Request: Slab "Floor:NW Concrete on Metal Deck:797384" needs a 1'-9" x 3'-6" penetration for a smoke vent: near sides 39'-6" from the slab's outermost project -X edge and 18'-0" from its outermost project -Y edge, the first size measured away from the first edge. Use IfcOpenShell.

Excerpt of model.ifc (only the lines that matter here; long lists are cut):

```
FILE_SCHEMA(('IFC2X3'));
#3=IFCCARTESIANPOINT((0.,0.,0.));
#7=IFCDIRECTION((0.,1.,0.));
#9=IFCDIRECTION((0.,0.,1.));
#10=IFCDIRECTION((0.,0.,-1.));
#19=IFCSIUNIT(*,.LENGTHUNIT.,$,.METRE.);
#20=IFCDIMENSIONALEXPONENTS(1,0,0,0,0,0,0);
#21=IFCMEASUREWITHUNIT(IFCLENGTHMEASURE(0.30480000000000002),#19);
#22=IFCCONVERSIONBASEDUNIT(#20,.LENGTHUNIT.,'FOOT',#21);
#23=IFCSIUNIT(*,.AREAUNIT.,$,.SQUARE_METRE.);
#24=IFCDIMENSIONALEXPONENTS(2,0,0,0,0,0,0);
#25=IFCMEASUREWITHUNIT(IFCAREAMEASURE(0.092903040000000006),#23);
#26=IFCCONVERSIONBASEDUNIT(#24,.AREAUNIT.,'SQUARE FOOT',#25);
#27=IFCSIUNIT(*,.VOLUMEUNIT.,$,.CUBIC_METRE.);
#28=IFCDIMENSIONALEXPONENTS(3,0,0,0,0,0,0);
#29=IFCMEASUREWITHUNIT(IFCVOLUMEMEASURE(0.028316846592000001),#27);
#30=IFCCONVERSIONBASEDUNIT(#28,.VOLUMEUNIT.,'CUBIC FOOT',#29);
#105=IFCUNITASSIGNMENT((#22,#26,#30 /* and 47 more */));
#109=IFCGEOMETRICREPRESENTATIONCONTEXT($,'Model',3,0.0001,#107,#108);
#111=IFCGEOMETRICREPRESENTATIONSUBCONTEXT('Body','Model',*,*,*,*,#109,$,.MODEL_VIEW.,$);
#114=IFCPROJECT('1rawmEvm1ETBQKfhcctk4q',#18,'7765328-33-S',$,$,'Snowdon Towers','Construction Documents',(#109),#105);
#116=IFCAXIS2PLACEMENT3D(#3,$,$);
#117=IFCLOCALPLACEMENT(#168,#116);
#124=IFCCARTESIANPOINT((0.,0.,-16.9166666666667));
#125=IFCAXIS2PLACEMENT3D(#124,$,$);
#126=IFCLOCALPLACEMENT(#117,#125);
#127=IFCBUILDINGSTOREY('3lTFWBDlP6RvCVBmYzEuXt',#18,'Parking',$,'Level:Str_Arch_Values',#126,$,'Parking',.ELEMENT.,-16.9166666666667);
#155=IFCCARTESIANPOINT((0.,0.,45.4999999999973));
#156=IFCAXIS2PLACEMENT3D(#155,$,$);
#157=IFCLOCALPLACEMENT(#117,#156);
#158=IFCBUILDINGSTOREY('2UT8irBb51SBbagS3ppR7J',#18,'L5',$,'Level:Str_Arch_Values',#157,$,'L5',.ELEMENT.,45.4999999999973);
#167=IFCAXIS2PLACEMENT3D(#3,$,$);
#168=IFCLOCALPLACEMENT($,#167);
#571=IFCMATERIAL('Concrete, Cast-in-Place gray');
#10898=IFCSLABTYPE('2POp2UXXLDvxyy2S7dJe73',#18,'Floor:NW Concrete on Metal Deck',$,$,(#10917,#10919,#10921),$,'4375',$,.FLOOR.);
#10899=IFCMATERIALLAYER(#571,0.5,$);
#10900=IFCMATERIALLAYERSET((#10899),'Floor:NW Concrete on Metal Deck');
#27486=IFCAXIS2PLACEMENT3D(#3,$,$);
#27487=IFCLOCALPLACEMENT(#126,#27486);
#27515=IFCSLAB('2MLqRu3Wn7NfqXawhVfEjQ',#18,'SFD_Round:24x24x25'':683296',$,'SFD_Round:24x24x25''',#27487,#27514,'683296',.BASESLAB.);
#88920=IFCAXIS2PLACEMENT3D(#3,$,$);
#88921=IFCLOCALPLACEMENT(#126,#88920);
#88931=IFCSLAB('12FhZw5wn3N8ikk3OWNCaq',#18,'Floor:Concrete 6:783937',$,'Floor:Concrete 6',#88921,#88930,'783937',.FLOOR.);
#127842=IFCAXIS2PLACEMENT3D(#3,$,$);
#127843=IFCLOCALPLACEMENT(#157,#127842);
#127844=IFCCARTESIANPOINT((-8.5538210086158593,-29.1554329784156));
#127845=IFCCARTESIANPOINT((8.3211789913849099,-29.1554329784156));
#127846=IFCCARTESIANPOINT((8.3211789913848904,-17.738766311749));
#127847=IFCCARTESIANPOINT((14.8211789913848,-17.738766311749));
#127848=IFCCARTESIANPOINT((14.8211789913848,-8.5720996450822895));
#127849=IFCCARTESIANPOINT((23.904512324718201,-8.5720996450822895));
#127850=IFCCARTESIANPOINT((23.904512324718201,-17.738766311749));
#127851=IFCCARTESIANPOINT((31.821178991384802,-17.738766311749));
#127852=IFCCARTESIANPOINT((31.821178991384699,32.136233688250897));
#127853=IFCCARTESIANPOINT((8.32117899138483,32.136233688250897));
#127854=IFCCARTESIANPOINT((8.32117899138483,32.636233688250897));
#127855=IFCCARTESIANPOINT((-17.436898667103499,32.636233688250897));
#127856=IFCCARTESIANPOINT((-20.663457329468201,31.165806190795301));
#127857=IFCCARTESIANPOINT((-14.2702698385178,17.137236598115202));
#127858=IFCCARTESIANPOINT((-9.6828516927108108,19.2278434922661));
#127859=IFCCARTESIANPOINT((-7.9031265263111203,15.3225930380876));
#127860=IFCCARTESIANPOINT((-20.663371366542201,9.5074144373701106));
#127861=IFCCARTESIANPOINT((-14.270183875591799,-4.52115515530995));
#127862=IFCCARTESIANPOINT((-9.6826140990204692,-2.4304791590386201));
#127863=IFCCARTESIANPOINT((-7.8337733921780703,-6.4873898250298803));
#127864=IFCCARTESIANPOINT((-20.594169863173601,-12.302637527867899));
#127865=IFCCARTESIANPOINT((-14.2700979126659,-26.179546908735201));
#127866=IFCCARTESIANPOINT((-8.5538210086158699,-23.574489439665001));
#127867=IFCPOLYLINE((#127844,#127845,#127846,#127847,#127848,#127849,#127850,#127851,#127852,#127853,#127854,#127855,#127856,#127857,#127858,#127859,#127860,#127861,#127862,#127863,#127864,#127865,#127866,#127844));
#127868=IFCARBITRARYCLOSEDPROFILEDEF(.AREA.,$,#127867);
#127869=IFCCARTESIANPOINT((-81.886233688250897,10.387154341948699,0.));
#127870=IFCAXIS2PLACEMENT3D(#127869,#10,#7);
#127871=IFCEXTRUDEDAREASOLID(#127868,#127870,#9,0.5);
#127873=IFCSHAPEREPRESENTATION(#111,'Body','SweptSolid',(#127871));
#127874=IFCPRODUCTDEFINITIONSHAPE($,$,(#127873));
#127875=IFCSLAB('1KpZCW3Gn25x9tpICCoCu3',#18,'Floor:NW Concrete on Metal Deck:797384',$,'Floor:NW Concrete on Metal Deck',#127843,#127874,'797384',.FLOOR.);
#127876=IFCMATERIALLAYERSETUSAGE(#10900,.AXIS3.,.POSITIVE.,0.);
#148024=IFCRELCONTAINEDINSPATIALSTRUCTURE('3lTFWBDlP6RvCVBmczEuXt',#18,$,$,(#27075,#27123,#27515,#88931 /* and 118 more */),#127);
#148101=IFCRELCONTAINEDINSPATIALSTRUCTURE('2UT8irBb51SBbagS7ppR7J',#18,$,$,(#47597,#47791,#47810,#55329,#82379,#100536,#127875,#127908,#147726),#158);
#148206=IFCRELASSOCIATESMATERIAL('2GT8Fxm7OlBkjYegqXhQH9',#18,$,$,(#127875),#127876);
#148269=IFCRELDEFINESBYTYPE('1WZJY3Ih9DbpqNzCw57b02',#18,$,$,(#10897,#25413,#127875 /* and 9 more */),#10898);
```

```python
import numpy as np
import ifcopenshell
import ifcopenshell.api.feature
import ifcopenshell.api.geometry
import ifcopenshell.api.root
import ifcopenshell.geom
import ifcopenshell.util.placement
import ifcopenshell.util.representation
import ifcopenshell.util.shape
import ifcopenshell.util.unit

model = ifcopenshell.open("model.ifc")
unit_scale = ifcopenshell.util.unit.calculate_unit_scale(model)
settings = ifcopenshell.geom.settings()


def volume(element):
    """Net volume in cubic metres, openings subtracted."""
    shape = ifcopenshell.geom.create_shape(settings, element)
    return ifcopenshell.util.shape.get_volume(shape.geometry)


slab = model.by_id(127875)
before = volume(slab)

# Extent in the slab's own axes, in metres. The edges named are its -X and -Y sides.
slab_shape = ifcopenshell.geom.create_shape(settings, slab)
vertices = ifcopenshell.util.shape.get_vertices(slab_shape.geometry)
x_min, y_min, bottom = vertices.min(axis=0)
top = vertices[:, 2].max()

opening = ifcopenshell.api.root.create_entity(model, ifc_class="IfcOpeningElement", name="Smoke vent opening")
context = ifcopenshell.util.representation.get_context(model, "Model", "Body", "MODEL_VIEW")
width, depth = 0.5334, 1.0668
outline = [(0.0, 0.0), (width, 0.0), (width, depth), (0.0, depth), (0.0, 0.0)]
# Overshoot both faces by 50 mm so the cut is clean.
shape = ifcopenshell.api.geometry.add_slab_representation(
    model, context=context, depth=top - bottom + 0.1, polyline=outline
)
ifcopenshell.api.geometry.assign_representation(model, product=opening, representation=shape)

matrix = ifcopenshell.util.placement.get_local_placement(slab.ObjectPlacement)
matrix[:, 3] = matrix @ np.append(np.array([x_min + 12.0396, y_min + 5.4864, bottom - 0.05]) / unit_scale, 1.0)
ifcopenshell.api.geometry.edit_object_placement(model, product=opening, matrix=matrix, is_si=False)
ifcopenshell.api.feature.add_feature(model, feature=opening, element=slab)

after = volume(slab)

print(f"slab volume {before:.3f} -> {after:.3f} m3")

model.write("model_updated.ifc")
```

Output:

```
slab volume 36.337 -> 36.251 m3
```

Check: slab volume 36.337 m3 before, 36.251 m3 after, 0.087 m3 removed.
